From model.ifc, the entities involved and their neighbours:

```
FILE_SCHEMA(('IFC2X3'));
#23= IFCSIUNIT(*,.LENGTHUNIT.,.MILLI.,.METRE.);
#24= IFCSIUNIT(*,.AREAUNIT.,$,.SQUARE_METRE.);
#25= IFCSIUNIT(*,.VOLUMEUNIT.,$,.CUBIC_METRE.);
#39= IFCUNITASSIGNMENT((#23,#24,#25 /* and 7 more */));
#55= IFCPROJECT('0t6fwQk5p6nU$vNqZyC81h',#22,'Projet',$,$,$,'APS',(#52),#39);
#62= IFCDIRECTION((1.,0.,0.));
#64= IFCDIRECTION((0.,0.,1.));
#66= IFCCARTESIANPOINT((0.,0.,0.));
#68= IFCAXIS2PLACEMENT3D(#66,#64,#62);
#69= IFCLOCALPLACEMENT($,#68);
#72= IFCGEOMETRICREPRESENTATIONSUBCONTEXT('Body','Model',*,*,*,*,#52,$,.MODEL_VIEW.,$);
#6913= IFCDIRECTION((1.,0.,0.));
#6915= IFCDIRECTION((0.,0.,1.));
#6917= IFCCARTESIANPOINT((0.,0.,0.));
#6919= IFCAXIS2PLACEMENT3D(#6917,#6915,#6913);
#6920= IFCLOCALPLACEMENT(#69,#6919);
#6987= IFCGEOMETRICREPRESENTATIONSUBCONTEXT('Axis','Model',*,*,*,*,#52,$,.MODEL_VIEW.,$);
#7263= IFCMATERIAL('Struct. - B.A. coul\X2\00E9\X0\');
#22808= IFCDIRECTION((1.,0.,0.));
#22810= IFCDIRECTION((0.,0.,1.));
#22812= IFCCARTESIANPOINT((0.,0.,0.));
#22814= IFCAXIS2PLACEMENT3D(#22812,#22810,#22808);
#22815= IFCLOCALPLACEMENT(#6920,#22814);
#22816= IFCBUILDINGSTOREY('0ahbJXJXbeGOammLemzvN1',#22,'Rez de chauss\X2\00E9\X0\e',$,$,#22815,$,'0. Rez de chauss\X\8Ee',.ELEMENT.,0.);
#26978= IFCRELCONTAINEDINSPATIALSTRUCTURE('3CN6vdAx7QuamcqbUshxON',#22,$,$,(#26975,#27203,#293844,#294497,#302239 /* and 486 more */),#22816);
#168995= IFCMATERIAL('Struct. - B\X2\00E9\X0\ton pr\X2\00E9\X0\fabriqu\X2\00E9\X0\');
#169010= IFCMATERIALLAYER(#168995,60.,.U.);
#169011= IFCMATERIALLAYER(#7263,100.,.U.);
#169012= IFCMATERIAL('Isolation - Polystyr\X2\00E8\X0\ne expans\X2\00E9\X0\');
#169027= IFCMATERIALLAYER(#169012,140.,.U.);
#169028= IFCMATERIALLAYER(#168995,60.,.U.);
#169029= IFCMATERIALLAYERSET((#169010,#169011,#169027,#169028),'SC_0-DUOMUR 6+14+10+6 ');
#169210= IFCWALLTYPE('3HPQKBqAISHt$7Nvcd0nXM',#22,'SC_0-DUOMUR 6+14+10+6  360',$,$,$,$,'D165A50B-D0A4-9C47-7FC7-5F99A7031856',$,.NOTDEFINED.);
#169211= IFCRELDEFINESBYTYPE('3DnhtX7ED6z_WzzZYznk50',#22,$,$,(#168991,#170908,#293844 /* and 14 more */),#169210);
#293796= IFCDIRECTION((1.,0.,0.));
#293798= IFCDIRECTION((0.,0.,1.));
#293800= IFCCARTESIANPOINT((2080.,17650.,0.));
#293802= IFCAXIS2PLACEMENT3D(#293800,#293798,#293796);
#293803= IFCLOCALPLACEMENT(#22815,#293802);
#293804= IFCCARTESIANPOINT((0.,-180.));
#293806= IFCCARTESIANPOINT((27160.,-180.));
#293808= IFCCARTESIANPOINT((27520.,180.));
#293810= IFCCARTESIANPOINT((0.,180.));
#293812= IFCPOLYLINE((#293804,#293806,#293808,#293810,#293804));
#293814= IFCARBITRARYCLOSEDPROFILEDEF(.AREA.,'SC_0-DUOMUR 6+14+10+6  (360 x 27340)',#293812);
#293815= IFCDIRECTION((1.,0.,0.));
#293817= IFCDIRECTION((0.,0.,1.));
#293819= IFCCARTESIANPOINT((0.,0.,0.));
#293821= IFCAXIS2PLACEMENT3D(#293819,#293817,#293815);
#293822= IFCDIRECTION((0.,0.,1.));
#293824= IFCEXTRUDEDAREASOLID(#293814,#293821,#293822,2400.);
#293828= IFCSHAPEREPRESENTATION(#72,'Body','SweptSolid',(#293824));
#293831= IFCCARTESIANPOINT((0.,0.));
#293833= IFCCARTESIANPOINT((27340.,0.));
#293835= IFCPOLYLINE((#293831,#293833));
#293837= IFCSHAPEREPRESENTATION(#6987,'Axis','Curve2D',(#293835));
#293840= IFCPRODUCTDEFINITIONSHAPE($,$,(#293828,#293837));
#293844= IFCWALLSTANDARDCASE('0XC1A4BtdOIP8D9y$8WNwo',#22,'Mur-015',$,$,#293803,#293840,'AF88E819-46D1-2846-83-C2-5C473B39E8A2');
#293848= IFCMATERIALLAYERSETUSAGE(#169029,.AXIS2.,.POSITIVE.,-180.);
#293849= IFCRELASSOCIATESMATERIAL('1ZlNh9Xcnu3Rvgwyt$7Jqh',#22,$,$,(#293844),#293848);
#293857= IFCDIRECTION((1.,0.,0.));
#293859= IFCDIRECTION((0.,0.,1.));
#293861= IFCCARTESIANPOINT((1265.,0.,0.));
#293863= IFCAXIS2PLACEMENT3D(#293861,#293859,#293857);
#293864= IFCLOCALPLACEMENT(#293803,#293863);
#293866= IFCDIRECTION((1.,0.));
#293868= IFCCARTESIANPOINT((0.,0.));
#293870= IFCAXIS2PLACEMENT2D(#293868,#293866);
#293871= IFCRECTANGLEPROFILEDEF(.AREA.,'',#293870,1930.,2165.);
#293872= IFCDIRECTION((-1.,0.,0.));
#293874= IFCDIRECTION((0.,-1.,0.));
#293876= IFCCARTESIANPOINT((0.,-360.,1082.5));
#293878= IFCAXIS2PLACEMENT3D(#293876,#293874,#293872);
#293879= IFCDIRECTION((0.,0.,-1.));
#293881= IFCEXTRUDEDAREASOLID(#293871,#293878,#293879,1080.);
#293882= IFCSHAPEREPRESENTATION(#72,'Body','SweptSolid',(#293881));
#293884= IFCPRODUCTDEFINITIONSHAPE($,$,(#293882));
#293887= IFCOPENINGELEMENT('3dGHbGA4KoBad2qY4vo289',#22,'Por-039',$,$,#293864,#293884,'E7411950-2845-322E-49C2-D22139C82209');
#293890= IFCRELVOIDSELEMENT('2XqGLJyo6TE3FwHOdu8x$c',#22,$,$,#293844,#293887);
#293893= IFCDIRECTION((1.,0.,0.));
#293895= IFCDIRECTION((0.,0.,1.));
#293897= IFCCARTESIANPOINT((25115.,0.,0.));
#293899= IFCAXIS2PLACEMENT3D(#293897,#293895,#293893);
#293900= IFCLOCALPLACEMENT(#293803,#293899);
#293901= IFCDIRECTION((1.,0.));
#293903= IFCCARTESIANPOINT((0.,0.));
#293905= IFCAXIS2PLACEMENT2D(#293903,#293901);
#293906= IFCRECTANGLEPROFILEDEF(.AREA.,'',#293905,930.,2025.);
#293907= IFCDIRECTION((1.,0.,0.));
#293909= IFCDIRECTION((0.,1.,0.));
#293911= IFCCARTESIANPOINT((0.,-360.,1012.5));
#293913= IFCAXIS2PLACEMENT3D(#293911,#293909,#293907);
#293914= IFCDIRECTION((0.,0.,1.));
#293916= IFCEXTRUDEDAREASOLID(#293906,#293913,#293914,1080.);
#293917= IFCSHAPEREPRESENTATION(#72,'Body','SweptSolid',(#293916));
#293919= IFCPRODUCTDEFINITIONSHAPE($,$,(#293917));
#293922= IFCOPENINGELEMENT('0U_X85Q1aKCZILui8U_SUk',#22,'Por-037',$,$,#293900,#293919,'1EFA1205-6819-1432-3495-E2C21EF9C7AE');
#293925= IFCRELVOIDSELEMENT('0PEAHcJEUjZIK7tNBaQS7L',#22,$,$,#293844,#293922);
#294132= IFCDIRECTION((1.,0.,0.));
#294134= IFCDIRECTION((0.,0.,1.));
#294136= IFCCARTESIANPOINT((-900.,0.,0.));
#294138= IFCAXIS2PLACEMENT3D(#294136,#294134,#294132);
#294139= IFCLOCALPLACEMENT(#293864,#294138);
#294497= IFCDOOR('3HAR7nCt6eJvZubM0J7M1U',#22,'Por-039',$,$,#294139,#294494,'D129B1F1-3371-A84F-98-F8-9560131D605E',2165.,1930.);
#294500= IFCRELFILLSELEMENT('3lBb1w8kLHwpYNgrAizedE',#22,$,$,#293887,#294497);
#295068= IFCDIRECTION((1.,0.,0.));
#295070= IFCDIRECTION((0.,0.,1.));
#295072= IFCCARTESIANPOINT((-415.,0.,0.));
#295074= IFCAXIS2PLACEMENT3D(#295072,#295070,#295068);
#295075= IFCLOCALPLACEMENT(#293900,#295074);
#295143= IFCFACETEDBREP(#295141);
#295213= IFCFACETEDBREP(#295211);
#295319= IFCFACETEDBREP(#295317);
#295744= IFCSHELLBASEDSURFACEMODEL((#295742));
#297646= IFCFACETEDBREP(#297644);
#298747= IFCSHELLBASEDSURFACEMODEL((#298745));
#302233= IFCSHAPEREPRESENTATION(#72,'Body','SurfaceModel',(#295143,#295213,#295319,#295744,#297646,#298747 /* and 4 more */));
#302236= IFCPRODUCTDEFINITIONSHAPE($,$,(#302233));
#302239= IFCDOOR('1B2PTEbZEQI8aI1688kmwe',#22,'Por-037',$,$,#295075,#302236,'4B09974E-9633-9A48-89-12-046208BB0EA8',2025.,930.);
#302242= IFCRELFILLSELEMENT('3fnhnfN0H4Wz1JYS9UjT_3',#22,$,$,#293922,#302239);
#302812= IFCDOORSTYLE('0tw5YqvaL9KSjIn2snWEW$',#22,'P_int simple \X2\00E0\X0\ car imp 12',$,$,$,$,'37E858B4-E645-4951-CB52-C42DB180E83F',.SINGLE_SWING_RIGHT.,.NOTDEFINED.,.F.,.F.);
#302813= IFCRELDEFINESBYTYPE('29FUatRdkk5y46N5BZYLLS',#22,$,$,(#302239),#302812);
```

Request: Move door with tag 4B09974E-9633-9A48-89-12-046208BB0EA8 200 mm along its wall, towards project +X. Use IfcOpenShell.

```python
import ifcopenshell
import ifcopenshell.api.geometry
import ifcopenshell.util.placement

model = ifcopenshell.open("model.ifc")

door = model.by_id(302239)
opening = door.FillsVoids[0].RelatingOpeningElement
wall = opening.VoidsElements[0].RelatingBuildingElement

wall_matrix = ifcopenshell.util.placement.get_local_placement(wall.ObjectPlacement)
shift = wall_matrix[:3, 0] * 200.0
before = ifcopenshell.util.placement.get_local_placement(door.ObjectPlacement)[:3, 3].copy()

# The door is placed relative to its opening, so it follows when the opening moves.
matrix = ifcopenshell.util.placement.get_local_placement(opening.ObjectPlacement)
matrix[:3, 3] += shift
ifcopenshell.api.geometry.edit_object_placement(
    model, product=opening, matrix=matrix, is_si=False, should_transform_children=True
)

after = ifcopenshell.util.placement.get_local_placement(door.ObjectPlacement)[:3, 3]
print("door moved by", (after - before).round(3) + 0.0)

model.write("model_rev.ifc")
```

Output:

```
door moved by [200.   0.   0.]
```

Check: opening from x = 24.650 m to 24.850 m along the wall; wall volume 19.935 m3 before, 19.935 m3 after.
